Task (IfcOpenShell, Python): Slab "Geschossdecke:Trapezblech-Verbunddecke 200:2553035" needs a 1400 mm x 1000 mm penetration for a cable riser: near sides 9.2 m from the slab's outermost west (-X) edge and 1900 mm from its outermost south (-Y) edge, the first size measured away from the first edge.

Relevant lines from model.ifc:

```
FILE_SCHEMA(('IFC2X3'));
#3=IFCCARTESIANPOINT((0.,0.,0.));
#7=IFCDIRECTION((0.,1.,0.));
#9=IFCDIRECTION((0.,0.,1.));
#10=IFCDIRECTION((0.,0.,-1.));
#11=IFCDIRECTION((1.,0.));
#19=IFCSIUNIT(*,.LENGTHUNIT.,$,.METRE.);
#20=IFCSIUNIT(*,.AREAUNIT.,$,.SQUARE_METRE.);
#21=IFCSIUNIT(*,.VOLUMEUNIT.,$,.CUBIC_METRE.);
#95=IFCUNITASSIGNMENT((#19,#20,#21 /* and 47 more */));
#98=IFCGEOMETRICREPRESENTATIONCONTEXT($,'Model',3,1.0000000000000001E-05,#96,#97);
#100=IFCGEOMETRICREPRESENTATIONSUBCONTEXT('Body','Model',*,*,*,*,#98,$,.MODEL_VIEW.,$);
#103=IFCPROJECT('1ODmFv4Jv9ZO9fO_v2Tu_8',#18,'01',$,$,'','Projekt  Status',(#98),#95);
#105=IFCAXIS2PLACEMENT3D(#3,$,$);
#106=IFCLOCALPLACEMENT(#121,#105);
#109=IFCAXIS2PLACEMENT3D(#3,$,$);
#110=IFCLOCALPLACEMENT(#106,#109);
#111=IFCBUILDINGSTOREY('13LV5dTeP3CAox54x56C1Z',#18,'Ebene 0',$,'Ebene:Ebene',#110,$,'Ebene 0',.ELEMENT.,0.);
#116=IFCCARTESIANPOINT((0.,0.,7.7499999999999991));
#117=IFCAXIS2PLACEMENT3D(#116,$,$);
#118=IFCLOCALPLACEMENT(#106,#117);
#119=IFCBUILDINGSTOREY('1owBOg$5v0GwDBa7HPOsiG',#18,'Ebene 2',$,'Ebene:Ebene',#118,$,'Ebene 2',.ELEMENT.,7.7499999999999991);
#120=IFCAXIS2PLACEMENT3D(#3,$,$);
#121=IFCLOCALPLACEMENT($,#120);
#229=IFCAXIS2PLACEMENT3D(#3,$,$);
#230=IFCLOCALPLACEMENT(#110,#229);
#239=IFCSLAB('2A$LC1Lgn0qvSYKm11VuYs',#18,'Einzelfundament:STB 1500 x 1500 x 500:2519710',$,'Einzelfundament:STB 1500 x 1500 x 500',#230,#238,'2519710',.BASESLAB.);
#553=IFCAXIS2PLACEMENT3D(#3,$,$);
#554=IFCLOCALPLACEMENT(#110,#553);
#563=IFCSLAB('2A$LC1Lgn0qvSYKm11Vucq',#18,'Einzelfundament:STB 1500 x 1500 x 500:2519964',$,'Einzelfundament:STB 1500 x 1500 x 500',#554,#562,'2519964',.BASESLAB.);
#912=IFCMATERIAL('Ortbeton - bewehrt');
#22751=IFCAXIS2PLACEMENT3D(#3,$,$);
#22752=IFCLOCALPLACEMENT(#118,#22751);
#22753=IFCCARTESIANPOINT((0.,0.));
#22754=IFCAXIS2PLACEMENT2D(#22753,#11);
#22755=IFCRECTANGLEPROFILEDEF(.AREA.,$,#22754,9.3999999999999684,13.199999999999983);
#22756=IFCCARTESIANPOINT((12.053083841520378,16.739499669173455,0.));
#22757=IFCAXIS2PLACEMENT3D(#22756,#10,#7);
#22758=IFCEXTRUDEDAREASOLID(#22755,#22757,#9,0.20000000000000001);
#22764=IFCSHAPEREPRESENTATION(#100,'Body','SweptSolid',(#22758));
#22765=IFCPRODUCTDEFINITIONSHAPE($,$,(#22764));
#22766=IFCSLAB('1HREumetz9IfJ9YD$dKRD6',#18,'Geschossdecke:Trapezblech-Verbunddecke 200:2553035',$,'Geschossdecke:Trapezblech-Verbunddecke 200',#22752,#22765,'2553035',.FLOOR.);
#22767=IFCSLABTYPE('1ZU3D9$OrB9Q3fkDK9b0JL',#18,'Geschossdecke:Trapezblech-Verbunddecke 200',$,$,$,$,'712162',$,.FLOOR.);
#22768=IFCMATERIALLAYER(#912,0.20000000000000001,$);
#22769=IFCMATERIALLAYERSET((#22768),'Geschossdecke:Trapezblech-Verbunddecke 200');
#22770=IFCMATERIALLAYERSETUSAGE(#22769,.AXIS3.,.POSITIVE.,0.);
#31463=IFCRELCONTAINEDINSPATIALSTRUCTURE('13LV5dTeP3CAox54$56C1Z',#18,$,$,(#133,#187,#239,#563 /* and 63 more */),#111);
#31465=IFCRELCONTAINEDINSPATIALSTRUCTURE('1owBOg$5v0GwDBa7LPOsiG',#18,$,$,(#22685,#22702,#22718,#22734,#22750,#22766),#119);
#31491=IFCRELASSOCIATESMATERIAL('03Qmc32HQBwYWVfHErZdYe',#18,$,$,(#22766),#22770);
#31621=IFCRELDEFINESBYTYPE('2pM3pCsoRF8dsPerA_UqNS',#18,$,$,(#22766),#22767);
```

```python
import numpy as np
import ifcopenshell
import ifcopenshell.api.feature
import ifcopenshell.api.geometry
import ifcopenshell.api.root
import ifcopenshell.geom
import ifcopenshell.util.placement
import ifcopenshell.util.representation
import ifcopenshell.util.shape
import ifcopenshell.util.unit

model = ifcopenshell.open("model.ifc")
unit_scale = ifcopenshell.util.unit.calculate_unit_scale(model)
settings = ifcopenshell.geom.settings()


def volume(element):
    """Net volume in cubic metres, openings subtracted."""
    shape = ifcopenshell.geom.create_shape(settings, element)
    return ifcopenshell.util.shape.get_volume(shape.geometry)


slab = model.by_id(22766)
before = volume(slab)

# Extent in the slab's own axes, in metres. The edges named are its -X and -Y sides.
slab_shape = ifcopenshell.geom.create_shape(settings, slab)
vertices = ifcopenshell.util.shape.get_vertices(slab_shape.geometry)
x_min, y_min, bottom = vertices.min(axis=0)
top = vertices[:, 2].max()

opening = ifcopenshell.api.root.create_entity(model, ifc_class="IfcOpeningElement", name="Cable riser opening")
context = ifcopenshell.util.representation.get_context(model, "Model", "Body", "MODEL_VIEW")
width, depth = 1.4, 1
outline = [(0.0, 0.0), (width, 0.0), (width, depth), (0.0, depth), (0.0, 0.0)]
# Overshoot both faces by 50 mm so the cut is clean.
shape = ifcopenshell.api.geometry.add_slab_representation(
    model, context=context, depth=top - bottom + 0.1, polyline=outline
)
ifcopenshell.api.geometry.assign_representation(model, product=opening, representation=shape)

matrix = ifcopenshell.util.placement.get_local_placement(slab.ObjectPlacement)
matrix[:, 3] = matrix @ np.append(np.array([x_min + 9.2, y_min + 1.9, bottom - 0.05]) / unit_scale, 1.0)
ifcopenshell.api.geometry.edit_object_placement(model, product=opening, matrix=matrix, is_si=False)
ifcopenshell.api.feature.add_feature(model, feature=opening, element=slab)

after = volume(slab)

print(f"slab volume {before:.3f} -> {after:.3f} m3")

model.write("model-out.ifc")
```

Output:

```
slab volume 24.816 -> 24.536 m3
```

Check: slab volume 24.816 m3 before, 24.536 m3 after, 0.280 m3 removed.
